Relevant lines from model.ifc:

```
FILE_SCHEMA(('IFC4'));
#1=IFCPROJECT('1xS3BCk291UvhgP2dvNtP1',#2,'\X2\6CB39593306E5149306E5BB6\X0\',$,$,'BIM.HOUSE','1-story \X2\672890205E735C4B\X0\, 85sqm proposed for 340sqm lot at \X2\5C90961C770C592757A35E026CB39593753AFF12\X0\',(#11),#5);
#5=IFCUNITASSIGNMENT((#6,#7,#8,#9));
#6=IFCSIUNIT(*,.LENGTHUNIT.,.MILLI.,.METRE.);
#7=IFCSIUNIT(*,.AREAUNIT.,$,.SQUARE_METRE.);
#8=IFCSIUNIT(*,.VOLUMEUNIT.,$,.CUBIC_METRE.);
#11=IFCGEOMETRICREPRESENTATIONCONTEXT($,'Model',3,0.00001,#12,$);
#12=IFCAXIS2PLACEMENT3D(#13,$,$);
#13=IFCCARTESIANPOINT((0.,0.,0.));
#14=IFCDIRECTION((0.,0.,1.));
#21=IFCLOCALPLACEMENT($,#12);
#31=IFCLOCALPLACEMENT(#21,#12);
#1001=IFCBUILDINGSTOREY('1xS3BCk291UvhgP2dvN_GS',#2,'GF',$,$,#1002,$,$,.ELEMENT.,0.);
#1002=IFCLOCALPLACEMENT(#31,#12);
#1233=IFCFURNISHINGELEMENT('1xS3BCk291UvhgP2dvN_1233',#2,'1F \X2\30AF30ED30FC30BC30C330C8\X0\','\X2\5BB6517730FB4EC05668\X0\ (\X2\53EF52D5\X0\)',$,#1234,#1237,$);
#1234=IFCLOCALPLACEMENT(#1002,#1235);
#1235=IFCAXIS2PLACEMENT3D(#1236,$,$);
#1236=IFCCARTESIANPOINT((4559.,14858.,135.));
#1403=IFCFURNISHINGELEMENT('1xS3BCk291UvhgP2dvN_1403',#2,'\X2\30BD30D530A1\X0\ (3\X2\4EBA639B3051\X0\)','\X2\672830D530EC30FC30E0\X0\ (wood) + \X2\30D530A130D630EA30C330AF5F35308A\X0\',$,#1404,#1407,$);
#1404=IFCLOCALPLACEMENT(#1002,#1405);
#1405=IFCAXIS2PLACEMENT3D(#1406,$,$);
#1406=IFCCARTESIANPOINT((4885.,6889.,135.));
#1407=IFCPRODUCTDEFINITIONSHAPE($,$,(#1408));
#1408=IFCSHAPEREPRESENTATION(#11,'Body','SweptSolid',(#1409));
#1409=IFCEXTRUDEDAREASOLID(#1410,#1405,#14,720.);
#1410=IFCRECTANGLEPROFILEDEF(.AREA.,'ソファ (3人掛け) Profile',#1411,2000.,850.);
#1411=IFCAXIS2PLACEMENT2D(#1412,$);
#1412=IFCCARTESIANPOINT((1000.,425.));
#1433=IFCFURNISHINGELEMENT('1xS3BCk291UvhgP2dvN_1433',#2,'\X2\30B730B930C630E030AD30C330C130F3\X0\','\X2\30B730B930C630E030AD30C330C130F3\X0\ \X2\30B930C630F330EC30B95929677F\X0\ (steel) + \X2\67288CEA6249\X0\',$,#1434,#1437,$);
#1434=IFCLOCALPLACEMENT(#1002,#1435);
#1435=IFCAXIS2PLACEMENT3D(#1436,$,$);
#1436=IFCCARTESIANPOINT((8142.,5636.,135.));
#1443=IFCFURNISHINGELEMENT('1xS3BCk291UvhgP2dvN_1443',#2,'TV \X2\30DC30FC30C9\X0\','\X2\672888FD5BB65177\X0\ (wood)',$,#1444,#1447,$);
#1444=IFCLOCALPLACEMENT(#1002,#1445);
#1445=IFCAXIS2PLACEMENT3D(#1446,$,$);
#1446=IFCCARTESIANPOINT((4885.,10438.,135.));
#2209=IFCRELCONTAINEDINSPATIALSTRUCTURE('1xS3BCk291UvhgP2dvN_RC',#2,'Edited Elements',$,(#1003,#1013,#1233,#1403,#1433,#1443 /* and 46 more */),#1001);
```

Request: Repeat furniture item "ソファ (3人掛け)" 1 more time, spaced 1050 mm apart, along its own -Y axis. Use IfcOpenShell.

```python
import ifcopenshell
import ifcopenshell.api.geometry
import ifcopenshell.api.root
import ifcopenshell.util.element
import ifcopenshell.util.placement
import ifcopenshell.util.unit

model = ifcopenshell.open("model.ifc")
unit_scale = ifcopenshell.util.unit.calculate_unit_scale(model)


def reuse_history(source, copy):
    """copy_class also copies each property set's owner history, people and application; keep the originals."""
    for rel in copy.IsDefinedBy:
        if rel.is_a("IfcRelDefinesByProperties") and (history := rel.RelatingPropertyDefinition.OwnerHistory):
            rel.RelatingPropertyDefinition.OwnerHistory = source.OwnerHistory
            ifcopenshell.util.element.remove_deep2(model, history)


source = model.by_id(1403)
base = ifcopenshell.util.placement.get_local_placement(source.ObjectPlacement)
step = -base[:3, 1] * 1.05 / unit_scale

for i in range(1, 2):
    copy = ifcopenshell.api.root.copy_class(model, product=source)
    copy.Representation = ifcopenshell.util.element.copy_deep(
        model, source.Representation, exclude=["IfcGeometricRepresentationContext", "IfcRepresentationMap"]
    )
    reuse_history(source, copy)
    matrix = base.copy()
    matrix[:3, 3] += i * step
    print("added at", matrix[:3, 3].round(3) + 0.0)
    ifcopenshell.api.geometry.edit_object_placement(model, product=copy, matrix=matrix, is_si=False)

model.write("model_rev.ifc")
```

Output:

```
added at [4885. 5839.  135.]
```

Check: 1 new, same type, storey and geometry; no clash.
